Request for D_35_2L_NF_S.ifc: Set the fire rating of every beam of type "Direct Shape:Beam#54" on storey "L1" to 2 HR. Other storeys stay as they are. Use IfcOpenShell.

First a look at what the model holds.

```python
import ifcopenshell
import ifcopenshell.util.element

model = ifcopenshell.open("D_35_2L_NF_S.ifc")
print(model.schema)
storey = next(s for s in model.by_type("IfcBuildingStorey") if s.Name == "L1")
beams = [e for e in ifcopenshell.util.element.get_decomposition(storey) if e.is_a("IfcBeam")]
seen = {}
for e in beams:
    element_type = ifcopenshell.util.element.get_type(e)
    key = (element_type.Name if element_type != e and element_type else None, ifcopenshell.util.element.get_pset(e, "Pset_BeamCommon", "FireRating"))
    seen[key] = seen.get(key, 0) + 1
for (name, value), count in sorted(seen.items(), key=str):
    print(count, "x", name, "|", value)
```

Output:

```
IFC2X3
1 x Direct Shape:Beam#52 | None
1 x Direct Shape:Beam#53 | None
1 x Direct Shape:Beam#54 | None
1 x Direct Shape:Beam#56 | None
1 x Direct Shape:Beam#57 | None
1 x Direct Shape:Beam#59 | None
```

```python
import ifcopenshell
import ifcopenshell.api.pset
import ifcopenshell.util.element

model = ifcopenshell.open("D_35_2L_NF_S.ifc")

storey = next(s for s in model.by_type("IfcBuildingStorey") if s.Name == "L1")
beams = [e for e in ifcopenshell.util.element.get_decomposition(storey) if e.is_a("IfcBeam")]

count = 0
for e in beams:
    element_type = ifcopenshell.util.element.get_type(e)
    if element_type in (None, e) or element_type.Name != "Direct Shape:Beam#54":
        continue
    # add_pset returns the element's existing set when there is one.
    pset = ifcopenshell.api.pset.add_pset(model, product=e, name="Pset_BeamCommon")
    ifcopenshell.api.pset.edit_pset(model, pset=pset, properties={"FireRating": "2 HR"})
    count += 1

print(count, "beams updated")

model.write("D_35_2L_NF_S_v2.ifc")
```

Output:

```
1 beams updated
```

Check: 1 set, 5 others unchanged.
